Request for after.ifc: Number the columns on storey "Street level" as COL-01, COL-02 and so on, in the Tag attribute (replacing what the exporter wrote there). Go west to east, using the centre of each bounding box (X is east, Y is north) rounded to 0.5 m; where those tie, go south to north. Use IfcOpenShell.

First a look at what the model holds.

```python
import ifcopenshell
import ifcopenshell.util.element
import ifcopenshell.util.placement

model = ifcopenshell.open("after.ifc")
print(model.schema)
storey = next(s for s in model.by_type("IfcBuildingStorey") if s.Name == "Street level")
columns = [e for e in ifcopenshell.util.element.get_decomposition(storey) if e.is_a("IfcColumn")]
for e in sorted(columns, key=lambda e: e.id()):
    origin = ifcopenshell.util.placement.get_local_placement(e.ObjectPlacement)[:3, 3]
    print(e.id(), e.Tag, e.Name, origin.round(2) + 0.0, sep=" | ")
```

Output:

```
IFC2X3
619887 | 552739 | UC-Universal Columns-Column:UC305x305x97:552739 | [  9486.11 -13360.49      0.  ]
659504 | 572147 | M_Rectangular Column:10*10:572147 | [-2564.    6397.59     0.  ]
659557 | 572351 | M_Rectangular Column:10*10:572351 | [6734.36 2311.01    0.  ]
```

```python
import ifcopenshell
import ifcopenshell.geom
import ifcopenshell.util.element
import ifcopenshell.util.shape

model = ifcopenshell.open("after.ifc")
settings = ifcopenshell.geom.settings()
settings.set("use-world-coords", True)


def centre(element):
    shape = ifcopenshell.geom.create_shape(settings, element)
    return ifcopenshell.util.shape.get_bbox_centroid(shape.geometry)


storey = next(s for s in model.by_type("IfcBuildingStorey") if s.Name == "Street level")
columns = [e for e in ifcopenshell.util.element.get_decomposition(storey) if e.is_a("IfcColumn")]

# Insertion points can sit at a corner or the storey origin, so sort by the geometry (in metres).
centres = {e: centre(e) for e in columns}
columns.sort(key=lambda e: (round(centres[e][0] / 0.5), centres[e][1]))

for i, e in enumerate(columns, start=1):
    number = f"COL-{i:02d}"
    e.Tag = number
    print(e.id(), number)

model.write("after_rev.ifc")
```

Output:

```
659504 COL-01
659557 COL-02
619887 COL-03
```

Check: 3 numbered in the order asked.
